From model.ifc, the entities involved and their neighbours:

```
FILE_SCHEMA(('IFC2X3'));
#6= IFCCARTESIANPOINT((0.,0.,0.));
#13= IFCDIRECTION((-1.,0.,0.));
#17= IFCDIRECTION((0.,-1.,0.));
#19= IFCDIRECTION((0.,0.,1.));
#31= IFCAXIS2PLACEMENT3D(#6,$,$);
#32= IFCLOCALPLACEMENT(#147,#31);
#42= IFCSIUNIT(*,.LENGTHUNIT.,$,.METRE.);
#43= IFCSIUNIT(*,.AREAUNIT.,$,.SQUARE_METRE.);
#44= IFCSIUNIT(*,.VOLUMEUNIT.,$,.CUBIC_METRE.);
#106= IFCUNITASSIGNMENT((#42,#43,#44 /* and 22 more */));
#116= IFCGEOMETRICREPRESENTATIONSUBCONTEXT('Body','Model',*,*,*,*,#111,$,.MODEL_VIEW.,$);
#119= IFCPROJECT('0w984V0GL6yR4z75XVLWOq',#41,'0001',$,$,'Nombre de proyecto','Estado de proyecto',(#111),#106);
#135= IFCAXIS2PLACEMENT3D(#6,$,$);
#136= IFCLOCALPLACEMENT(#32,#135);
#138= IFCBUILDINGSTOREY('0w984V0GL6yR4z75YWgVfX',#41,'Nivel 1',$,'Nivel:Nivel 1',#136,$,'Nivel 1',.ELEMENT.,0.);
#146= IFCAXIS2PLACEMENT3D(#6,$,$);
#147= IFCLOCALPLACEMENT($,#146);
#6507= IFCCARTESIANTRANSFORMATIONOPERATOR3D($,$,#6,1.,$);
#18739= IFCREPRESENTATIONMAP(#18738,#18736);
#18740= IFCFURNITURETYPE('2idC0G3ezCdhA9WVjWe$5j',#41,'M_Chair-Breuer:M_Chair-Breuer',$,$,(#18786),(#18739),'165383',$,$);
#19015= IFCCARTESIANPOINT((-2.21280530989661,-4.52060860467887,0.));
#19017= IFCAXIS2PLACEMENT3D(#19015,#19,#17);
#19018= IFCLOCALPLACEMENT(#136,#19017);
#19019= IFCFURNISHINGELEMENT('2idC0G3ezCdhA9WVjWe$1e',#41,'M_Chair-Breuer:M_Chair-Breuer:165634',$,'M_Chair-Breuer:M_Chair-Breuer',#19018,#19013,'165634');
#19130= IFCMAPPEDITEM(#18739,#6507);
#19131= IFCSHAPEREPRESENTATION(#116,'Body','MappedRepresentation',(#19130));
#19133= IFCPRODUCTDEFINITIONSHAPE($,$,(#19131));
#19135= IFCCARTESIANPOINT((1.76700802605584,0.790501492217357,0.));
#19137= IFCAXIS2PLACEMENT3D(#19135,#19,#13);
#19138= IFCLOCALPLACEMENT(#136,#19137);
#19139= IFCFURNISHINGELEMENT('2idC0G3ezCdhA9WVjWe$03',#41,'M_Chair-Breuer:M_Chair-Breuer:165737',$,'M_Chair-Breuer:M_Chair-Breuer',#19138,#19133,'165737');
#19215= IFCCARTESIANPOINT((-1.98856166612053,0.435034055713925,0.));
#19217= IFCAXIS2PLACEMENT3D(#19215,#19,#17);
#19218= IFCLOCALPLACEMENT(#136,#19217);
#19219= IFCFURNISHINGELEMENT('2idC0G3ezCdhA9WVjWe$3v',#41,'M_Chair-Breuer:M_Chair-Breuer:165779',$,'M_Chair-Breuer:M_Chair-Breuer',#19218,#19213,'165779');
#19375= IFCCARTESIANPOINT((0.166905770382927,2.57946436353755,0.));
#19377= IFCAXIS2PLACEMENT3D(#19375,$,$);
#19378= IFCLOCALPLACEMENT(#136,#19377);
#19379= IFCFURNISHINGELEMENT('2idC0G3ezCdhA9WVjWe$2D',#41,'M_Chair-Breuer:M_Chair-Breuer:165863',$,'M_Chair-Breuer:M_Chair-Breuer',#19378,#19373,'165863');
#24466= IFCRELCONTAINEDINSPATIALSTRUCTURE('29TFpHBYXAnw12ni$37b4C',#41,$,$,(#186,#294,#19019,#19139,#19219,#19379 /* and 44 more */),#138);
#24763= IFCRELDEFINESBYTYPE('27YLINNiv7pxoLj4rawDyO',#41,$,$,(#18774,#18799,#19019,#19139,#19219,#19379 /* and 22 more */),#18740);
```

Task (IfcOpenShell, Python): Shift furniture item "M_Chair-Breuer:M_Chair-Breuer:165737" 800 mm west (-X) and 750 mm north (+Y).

```python
import ifcopenshell
import ifcopenshell.api.geometry
import ifcopenshell.util.placement
import ifcopenshell.util.unit

model = ifcopenshell.open("model.ifc")
unit_scale = ifcopenshell.util.unit.calculate_unit_scale(model)

item = model.by_guid("2idC0G3ezCdhA9WVjWe$03")
matrix = ifcopenshell.util.placement.get_local_placement(item.ObjectPlacement)
matrix[0, 3] -= 0.8 / unit_scale
matrix[1, 3] += 0.75 / unit_scale
ifcopenshell.api.geometry.edit_object_placement(model, product=item, matrix=matrix, is_si=False)

print(ifcopenshell.util.placement.get_local_placement(item.ObjectPlacement).round(3) + 0.0)

model.write("model-out.ifc")
```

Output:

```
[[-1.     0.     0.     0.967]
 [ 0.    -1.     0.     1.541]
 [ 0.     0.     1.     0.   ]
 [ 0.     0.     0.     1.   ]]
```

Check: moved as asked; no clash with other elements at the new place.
